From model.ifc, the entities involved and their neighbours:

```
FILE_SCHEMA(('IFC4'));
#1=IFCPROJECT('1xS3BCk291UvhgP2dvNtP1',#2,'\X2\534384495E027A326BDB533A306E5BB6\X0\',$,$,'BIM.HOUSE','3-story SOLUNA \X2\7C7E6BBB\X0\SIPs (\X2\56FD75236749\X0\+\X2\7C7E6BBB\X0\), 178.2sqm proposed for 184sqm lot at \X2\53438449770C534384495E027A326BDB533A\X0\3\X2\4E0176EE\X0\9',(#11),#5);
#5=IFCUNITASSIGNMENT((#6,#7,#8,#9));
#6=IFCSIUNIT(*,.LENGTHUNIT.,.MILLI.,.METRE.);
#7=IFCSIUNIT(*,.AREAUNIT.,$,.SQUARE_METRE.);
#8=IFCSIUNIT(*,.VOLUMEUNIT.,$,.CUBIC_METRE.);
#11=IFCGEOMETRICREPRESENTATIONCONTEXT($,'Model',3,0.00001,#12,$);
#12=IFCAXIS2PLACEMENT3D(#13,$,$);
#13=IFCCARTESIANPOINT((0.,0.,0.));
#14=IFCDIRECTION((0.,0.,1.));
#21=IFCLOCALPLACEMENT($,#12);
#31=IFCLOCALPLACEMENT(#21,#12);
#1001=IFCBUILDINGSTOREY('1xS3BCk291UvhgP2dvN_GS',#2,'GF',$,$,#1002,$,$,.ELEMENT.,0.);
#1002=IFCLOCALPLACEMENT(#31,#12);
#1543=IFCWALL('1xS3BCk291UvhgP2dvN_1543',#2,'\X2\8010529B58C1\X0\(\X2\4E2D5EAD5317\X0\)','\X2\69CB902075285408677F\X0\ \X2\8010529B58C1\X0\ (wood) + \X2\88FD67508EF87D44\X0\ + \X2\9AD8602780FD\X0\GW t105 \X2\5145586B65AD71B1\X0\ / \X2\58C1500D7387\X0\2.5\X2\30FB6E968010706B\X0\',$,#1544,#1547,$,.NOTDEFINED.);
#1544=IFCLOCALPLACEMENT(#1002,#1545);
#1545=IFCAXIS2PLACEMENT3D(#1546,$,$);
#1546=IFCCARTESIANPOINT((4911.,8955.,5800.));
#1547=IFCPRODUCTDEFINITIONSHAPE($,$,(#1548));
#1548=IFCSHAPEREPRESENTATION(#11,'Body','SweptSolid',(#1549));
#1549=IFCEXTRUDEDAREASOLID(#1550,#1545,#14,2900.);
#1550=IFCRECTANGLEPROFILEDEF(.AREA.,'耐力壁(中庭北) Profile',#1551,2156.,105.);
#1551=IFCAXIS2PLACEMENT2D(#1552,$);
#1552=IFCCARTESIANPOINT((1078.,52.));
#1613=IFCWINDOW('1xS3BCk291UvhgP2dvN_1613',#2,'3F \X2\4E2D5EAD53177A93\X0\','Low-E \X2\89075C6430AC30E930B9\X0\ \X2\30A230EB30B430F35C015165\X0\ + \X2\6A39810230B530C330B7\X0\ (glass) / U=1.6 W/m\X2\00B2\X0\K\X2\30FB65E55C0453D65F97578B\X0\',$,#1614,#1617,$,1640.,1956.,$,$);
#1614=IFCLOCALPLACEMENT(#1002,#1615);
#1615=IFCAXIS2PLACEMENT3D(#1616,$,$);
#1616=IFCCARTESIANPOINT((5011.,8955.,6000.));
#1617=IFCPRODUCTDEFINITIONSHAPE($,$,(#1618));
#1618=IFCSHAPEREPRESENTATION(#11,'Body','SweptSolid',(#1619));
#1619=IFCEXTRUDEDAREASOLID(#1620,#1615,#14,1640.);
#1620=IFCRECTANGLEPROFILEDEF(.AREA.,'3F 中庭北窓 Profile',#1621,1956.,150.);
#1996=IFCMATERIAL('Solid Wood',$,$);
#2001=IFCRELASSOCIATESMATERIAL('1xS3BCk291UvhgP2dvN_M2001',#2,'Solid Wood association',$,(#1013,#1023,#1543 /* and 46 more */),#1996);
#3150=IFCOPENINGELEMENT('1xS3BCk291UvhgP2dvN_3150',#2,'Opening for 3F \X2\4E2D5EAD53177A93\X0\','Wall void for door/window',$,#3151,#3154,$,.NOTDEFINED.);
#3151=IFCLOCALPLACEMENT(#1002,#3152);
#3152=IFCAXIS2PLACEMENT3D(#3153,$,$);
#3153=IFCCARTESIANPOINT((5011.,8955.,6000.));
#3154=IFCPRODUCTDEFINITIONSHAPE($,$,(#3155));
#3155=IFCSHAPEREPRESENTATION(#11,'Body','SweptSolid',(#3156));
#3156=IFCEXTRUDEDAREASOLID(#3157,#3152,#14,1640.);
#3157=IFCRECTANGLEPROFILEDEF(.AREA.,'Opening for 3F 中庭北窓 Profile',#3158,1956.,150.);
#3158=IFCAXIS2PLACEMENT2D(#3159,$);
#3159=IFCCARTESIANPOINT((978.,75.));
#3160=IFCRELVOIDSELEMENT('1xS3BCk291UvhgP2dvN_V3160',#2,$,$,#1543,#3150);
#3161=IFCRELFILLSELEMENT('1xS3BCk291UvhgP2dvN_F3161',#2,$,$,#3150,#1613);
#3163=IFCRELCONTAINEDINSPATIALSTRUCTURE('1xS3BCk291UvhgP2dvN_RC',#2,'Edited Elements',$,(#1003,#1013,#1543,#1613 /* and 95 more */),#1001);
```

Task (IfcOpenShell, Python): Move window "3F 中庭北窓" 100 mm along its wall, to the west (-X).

```python
import ifcopenshell
import ifcopenshell.api.geometry
import ifcopenshell.util.placement

model = ifcopenshell.open("model.ifc")

window = model.by_id(1613)
opening = window.FillsVoids[0].RelatingOpeningElement
wall = opening.VoidsElements[0].RelatingBuildingElement

wall_matrix = ifcopenshell.util.placement.get_local_placement(wall.ObjectPlacement)
shift = wall_matrix[:3, 0] * -100.0
before = ifcopenshell.util.placement.get_local_placement(window.ObjectPlacement)[:3, 3].copy()

# The window is not placed relative to its opening, so move both.
for product in (opening, window):
    matrix = ifcopenshell.util.placement.get_local_placement(product.ObjectPlacement)
    matrix[:3, 3] += shift
    ifcopenshell.api.geometry.edit_object_placement(model, product=product, matrix=matrix, is_si=False)

after = ifcopenshell.util.placement.get_local_placement(window.ObjectPlacement)[:3, 3]
print("window moved by", (after - before).round(3) + 0.0)

model.write("model_v2.ifc")
```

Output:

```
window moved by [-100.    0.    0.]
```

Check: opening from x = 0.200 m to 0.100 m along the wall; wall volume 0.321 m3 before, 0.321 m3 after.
